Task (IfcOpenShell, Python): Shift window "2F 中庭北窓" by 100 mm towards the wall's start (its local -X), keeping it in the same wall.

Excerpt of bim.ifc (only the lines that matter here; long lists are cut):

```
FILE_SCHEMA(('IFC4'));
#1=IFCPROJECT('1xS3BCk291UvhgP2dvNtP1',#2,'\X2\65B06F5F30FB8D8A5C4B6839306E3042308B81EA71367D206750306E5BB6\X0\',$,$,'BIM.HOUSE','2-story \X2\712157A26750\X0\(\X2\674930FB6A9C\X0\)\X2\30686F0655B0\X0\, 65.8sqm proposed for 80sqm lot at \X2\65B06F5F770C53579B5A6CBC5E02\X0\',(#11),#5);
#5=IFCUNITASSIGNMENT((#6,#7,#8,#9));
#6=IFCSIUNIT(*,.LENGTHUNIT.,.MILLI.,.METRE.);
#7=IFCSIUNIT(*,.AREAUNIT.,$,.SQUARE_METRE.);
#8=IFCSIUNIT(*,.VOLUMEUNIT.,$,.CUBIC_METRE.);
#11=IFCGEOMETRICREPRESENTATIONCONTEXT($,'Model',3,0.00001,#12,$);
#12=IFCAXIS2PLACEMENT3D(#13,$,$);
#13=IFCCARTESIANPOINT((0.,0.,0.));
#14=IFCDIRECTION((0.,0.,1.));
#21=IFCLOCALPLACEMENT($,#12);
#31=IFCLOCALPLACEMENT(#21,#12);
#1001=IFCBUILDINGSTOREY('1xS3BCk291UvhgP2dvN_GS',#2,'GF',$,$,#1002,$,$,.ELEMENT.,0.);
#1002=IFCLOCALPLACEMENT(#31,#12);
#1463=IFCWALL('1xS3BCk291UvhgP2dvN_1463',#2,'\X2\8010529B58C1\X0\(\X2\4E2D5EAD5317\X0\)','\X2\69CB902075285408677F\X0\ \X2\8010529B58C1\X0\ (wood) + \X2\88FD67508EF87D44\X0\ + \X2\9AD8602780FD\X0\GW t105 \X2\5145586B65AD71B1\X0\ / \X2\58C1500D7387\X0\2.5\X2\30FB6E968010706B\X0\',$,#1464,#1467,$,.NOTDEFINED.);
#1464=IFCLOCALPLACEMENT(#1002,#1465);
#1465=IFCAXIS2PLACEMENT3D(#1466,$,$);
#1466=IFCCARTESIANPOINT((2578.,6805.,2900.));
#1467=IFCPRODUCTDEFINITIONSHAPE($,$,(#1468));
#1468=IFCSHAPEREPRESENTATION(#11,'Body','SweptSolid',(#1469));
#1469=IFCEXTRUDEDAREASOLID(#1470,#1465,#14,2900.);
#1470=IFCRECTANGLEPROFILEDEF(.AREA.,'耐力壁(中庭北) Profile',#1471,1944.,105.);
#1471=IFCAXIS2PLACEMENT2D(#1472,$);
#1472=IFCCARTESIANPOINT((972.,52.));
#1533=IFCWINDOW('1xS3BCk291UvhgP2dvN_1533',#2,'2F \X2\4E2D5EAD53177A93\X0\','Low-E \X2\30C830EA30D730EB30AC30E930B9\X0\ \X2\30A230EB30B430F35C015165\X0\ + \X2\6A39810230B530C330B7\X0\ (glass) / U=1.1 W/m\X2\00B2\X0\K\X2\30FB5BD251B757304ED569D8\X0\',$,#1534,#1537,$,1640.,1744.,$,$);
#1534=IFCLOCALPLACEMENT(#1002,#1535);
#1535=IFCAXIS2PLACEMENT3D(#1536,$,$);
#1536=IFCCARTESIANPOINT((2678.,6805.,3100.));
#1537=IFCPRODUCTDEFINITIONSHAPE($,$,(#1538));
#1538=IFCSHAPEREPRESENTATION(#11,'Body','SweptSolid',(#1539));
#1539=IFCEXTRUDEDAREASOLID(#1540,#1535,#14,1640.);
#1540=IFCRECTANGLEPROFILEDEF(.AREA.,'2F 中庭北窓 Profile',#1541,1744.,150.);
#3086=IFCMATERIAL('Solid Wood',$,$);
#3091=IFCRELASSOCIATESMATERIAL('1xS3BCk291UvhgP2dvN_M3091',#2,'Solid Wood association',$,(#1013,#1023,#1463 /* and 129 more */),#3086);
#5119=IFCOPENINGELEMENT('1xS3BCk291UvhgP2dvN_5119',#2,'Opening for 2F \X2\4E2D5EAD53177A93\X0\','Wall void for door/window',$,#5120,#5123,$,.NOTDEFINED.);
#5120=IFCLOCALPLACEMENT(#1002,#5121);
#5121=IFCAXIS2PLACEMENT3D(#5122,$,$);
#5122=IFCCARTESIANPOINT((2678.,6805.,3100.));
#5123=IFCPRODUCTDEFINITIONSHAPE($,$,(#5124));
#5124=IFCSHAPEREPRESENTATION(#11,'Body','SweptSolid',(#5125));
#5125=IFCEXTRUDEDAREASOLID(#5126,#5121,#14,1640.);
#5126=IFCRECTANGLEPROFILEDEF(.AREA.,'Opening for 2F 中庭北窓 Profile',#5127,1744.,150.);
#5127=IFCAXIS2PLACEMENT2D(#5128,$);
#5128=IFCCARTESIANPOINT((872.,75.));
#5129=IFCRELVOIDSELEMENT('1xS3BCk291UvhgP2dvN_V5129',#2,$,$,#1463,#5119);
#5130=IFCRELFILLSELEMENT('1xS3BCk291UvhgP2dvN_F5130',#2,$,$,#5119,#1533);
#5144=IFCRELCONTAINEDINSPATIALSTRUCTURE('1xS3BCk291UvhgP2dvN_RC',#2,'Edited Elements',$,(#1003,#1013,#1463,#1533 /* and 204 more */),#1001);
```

```python
import ifcopenshell
import ifcopenshell.api.geometry
import ifcopenshell.util.placement

model = ifcopenshell.open("bim.ifc")

window = model.by_id(1533)
opening = window.FillsVoids[0].RelatingOpeningElement
wall = opening.VoidsElements[0].RelatingBuildingElement

wall_matrix = ifcopenshell.util.placement.get_local_placement(wall.ObjectPlacement)
shift = wall_matrix[:3, 0] * -100.0
before = ifcopenshell.util.placement.get_local_placement(window.ObjectPlacement)[:3, 3].copy()

# The window is not placed relative to its opening, so move both.
for product in (opening, window):
    matrix = ifcopenshell.util.placement.get_local_placement(product.ObjectPlacement)
    matrix[:3, 3] += shift
    ifcopenshell.api.geometry.edit_object_placement(model, product=product, matrix=matrix, is_si=False)

after = ifcopenshell.util.placement.get_local_placement(window.ObjectPlacement)[:3, 3]
print("window moved by", (after - before).round(3) + 0.0)

model.write("bim_rev.ifc")
```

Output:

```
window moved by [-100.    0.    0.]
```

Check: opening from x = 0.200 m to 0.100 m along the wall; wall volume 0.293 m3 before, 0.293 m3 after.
